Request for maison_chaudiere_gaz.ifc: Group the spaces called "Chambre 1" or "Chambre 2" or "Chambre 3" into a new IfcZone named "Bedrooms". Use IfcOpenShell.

First a look at what the model holds.

```python
import ifcopenshell

model = ifcopenshell.open("maison_chaudiere_gaz.ifc")
print(model.schema)
seen = {}
for space in model.by_type("IfcSpace"):
    seen[space.LongName] = seen.get(space.LongName, 0) + 1
for name, count in sorted(seen.items(), key=str):
    print(count, "x", name)
print("zones:", [z.Name for z in model.by_type("IfcZone")][:20])
```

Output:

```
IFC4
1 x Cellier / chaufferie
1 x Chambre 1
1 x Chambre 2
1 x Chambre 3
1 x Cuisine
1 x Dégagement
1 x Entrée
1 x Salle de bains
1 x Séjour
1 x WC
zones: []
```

```python
import ifcopenshell
import ifcopenshell.api.group
import ifcopenshell.api.root

model = ifcopenshell.open("maison_chaudiere_gaz.ifc")

names = {"Chambre 1", "Chambre 2", "Chambre 3"}
spaces = [s for s in model.by_type("IfcSpace") if s.LongName in names]

zone = ifcopenshell.api.root.create_entity(model, ifc_class="IfcZone", name="Bedrooms")
ifcopenshell.api.group.assign_group(model, products=spaces, group=zone)
print(len(spaces), "spaces in", zone.Name)

model.write("maison_chaudiere_gaz_updated.ifc")
```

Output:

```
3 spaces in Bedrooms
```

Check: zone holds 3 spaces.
